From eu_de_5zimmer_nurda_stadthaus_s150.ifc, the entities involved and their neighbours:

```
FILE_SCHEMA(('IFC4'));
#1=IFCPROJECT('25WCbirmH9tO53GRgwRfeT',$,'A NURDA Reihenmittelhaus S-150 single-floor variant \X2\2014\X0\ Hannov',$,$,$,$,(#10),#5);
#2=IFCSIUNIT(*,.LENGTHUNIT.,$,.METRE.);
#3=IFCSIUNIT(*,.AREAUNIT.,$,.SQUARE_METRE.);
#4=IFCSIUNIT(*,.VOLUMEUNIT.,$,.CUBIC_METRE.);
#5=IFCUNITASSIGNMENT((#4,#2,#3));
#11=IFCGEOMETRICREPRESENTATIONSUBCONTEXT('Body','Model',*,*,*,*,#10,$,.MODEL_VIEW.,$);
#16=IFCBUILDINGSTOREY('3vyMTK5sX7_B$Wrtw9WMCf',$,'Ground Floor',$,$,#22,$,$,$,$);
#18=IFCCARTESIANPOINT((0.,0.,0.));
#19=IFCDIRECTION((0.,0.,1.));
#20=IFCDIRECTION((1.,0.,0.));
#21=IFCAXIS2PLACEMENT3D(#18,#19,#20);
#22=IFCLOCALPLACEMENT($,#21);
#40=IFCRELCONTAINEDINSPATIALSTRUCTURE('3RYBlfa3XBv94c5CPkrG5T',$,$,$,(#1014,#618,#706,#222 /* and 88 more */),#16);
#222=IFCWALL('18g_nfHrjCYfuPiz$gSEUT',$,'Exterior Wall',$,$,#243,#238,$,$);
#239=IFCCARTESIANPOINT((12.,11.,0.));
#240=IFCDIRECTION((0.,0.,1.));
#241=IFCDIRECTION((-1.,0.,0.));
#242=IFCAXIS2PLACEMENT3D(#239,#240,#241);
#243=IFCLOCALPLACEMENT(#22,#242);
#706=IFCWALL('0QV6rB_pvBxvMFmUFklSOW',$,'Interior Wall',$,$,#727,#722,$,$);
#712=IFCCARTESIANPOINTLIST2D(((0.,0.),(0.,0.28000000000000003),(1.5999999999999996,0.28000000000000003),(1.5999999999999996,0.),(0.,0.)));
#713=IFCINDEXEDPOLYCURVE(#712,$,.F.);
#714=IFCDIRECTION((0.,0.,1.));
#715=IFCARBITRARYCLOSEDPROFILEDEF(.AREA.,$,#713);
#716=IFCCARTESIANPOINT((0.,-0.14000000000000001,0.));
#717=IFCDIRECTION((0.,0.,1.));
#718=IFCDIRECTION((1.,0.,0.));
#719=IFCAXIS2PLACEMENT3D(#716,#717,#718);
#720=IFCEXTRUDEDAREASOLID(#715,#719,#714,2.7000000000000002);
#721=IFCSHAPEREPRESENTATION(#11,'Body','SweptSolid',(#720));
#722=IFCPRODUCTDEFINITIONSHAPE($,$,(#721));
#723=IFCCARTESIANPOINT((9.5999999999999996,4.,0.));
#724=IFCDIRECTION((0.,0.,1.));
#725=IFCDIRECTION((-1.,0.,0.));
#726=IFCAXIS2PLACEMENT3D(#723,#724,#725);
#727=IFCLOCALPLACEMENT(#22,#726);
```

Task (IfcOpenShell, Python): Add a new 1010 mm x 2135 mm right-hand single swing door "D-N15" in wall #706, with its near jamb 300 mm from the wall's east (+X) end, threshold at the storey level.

```python
import numpy as np
import ifcopenshell
import ifcopenshell.api.feature
import ifcopenshell.api.geometry
import ifcopenshell.api.root
import ifcopenshell.api.spatial
import ifcopenshell.geom
import ifcopenshell.util.element
import ifcopenshell.util.placement
import ifcopenshell.util.representation
import ifcopenshell.util.shape
import ifcopenshell.util.unit

model = ifcopenshell.open("eu_de_5zimmer_nurda_stadthaus_s150.ifc")
unit_scale = ifcopenshell.util.unit.calculate_unit_scale(model)
settings = ifcopenshell.geom.settings()


def volume(element):
    """Net volume in cubic metres, openings subtracted."""
    shape = ifcopenshell.geom.create_shape(settings, element)
    return ifcopenshell.util.shape.get_volume(shape.geometry)


wall = model.by_guid("0QV6rB_pvBxvMFmUFklSOW")
storey = ifcopenshell.util.element.get_container(wall, ifc_class="IfcBuildingStorey")
context = ifcopenshell.util.representation.get_context(model, "Model", "Body", "MODEL_VIEW")
before = volume(wall)

width, height, from_end, sill = 1.01, 2.135, 0.3, 0.0  # metres

# The wall runs along its own X axis, and the end named is its -X end.
wall_shape = ifcopenshell.geom.create_shape(settings, wall)
x, y, z = ifcopenshell.util.shape.get_vertices(wall_shape.geometry).T
start = x.min() + from_end
face, thickness = float(y.min()), float(y.max() - y.min())
wall_matrix = ifcopenshell.util.placement.get_local_placement(wall.ObjectPlacement)
level = ifcopenshell.util.placement.get_local_placement(storey.ObjectPlacement)[2, 3]


def in_wall(x, y):
    """Placement at x, y metres in the wall's axes, at sill height."""
    matrix = wall_matrix.copy()
    matrix[:, 3] = wall_matrix @ np.array([x / unit_scale, y / unit_scale, 0.0, 1.0])
    matrix[2, 3] = level + sill / unit_scale
    return matrix


# Opening: a box that overshoots both wall faces by 50 mm.
opening = ifcopenshell.api.root.create_entity(model, ifc_class="IfcOpeningElement", predefined_type="OPENING")
box = ifcopenshell.api.geometry.add_wall_representation(
    model, context=context, length=width, height=height, thickness=thickness + 0.1
)
ifcopenshell.api.geometry.assign_representation(model, product=opening, representation=box)
ifcopenshell.api.geometry.edit_object_placement(model, product=opening, matrix=in_wall(start, face - 0.05), is_si=False)
ifcopenshell.api.feature.add_feature(model, feature=opening, element=wall)

door = ifcopenshell.api.root.create_entity(model, ifc_class="IfcDoor", name="D-N15", predefined_type="DOOR")
door.OverallWidth, door.OverallHeight = width / unit_scale, height / unit_scale
door.OperationType = "SINGLE_SWING_RIGHT"
body = ifcopenshell.api.geometry.add_door_representation(
    model,
    context=context,
    overall_width=door.OverallWidth,
    overall_height=door.OverallHeight,
    operation_type="SINGLE_SWING_RIGHT",
    lining_properties={"LiningDepth": thickness / unit_scale, "ThresholdDepth": thickness / unit_scale},
)
ifcopenshell.api.geometry.assign_representation(model, product=door, representation=body)
ifcopenshell.api.spatial.assign_container(model, products=[door], relating_structure=storey)
ifcopenshell.api.feature.add_filling(model, opening=opening, element=door)

# The lining spans the wall, so the door starts at the wall face.
ifcopenshell.api.geometry.edit_object_placement(model, product=door, matrix=in_wall(start, face), is_si=False)

after = volume(wall)

print(f"wall volume {before:.3f} -> {after:.3f} m3")

model.write("eu_de_5zimmer_nurda_stadthaus_s150_edited.ifc")
```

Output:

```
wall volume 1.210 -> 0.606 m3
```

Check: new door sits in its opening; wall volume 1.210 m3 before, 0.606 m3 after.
